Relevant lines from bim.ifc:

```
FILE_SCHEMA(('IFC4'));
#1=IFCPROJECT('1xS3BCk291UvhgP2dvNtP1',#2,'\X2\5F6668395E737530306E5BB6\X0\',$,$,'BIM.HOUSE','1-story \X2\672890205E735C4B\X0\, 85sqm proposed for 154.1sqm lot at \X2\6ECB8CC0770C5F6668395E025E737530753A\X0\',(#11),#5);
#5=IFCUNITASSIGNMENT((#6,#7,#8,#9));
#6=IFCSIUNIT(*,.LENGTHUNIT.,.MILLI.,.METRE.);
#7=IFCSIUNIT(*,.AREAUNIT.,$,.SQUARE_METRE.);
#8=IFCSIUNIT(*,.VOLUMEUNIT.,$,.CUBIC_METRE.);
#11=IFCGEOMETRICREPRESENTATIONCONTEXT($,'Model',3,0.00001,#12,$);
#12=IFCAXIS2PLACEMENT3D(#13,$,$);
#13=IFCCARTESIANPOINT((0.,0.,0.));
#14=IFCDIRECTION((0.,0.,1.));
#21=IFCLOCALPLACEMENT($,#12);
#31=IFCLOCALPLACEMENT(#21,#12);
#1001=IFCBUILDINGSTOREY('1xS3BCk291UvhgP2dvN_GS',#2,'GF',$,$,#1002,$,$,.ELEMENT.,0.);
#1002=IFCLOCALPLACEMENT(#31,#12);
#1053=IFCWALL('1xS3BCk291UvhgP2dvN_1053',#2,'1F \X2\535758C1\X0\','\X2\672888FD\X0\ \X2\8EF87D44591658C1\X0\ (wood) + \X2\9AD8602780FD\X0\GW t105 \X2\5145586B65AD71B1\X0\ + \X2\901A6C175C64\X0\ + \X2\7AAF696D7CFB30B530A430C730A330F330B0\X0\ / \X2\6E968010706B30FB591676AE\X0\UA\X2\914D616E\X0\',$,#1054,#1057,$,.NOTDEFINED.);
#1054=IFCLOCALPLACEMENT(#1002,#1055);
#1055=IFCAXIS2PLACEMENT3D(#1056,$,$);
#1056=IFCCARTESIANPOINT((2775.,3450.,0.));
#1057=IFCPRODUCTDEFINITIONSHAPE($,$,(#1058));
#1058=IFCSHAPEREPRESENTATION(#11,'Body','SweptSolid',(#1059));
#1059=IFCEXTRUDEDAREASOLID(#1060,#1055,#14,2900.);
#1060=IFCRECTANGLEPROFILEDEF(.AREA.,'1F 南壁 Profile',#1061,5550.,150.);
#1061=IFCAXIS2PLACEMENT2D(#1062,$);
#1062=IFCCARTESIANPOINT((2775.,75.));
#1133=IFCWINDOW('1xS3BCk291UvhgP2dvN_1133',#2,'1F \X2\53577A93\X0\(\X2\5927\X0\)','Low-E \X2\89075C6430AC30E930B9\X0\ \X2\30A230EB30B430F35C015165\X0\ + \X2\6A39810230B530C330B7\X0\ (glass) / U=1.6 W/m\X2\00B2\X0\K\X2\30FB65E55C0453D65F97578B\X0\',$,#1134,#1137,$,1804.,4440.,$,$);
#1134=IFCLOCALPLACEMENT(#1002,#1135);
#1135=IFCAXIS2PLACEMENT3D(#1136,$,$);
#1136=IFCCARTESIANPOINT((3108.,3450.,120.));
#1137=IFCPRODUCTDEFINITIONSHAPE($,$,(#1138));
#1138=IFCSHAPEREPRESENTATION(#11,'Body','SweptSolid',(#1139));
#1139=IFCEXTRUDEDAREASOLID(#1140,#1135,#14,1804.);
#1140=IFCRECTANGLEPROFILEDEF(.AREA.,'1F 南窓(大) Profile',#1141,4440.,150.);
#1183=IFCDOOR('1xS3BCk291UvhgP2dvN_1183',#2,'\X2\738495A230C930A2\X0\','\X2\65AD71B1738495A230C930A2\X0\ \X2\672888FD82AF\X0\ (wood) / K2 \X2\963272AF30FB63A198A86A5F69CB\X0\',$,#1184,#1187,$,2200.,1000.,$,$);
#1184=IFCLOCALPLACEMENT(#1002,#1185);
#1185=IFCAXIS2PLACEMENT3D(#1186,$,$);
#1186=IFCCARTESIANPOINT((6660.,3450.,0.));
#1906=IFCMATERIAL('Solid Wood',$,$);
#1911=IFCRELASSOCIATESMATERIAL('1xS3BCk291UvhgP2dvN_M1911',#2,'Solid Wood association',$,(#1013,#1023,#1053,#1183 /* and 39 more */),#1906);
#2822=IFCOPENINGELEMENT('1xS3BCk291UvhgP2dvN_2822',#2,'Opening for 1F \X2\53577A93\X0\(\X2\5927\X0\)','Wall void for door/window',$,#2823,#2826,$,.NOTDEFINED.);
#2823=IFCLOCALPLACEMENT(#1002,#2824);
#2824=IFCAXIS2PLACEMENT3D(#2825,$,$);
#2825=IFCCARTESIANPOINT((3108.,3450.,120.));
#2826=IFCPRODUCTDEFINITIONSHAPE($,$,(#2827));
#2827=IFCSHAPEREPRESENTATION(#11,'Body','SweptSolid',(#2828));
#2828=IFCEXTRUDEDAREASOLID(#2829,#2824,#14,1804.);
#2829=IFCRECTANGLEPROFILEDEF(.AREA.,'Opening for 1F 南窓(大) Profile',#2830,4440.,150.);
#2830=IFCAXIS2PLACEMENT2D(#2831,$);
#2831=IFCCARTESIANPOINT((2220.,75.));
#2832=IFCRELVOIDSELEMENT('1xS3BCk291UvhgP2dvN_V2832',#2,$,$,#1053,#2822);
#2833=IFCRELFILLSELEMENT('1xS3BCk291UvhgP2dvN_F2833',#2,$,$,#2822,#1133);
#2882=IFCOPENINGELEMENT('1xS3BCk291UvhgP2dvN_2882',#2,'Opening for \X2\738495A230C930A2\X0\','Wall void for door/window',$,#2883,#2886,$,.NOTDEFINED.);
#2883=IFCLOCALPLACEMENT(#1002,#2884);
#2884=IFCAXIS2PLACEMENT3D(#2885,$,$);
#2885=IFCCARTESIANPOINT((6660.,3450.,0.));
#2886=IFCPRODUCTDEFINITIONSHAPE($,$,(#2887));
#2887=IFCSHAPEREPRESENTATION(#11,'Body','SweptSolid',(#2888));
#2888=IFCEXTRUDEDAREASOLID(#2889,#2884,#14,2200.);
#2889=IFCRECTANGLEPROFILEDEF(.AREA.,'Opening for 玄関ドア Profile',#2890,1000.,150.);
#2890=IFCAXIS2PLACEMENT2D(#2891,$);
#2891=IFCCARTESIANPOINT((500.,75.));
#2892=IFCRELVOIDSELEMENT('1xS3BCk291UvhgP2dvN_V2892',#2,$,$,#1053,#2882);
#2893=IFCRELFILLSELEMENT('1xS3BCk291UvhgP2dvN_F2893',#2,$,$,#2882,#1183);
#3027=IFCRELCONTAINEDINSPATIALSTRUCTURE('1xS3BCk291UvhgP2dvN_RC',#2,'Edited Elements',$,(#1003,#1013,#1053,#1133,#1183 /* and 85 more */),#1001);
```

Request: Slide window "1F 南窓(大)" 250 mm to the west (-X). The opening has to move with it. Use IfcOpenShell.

```python
import ifcopenshell
import ifcopenshell.api.geometry
import ifcopenshell.util.placement

model = ifcopenshell.open("bim.ifc")

window = model.by_id(1133)
opening = window.FillsVoids[0].RelatingOpeningElement
wall = opening.VoidsElements[0].RelatingBuildingElement

wall_matrix = ifcopenshell.util.placement.get_local_placement(wall.ObjectPlacement)
shift = wall_matrix[:3, 0] * -250.0
before = ifcopenshell.util.placement.get_local_placement(window.ObjectPlacement)[:3, 3].copy()

# The window is not placed relative to its opening, so move both.
for product in (opening, window):
    matrix = ifcopenshell.util.placement.get_local_placement(product.ObjectPlacement)
    matrix[:3, 3] += shift
    ifcopenshell.api.geometry.edit_object_placement(model, product=product, matrix=matrix, is_si=False)

after = ifcopenshell.util.placement.get_local_placement(window.ObjectPlacement)[:3, 3]
print("window moved by", (after - before).round(3) + 0.0)

model.write("bim_edited.ifc")
```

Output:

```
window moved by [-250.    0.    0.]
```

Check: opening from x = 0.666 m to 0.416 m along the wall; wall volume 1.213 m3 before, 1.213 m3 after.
